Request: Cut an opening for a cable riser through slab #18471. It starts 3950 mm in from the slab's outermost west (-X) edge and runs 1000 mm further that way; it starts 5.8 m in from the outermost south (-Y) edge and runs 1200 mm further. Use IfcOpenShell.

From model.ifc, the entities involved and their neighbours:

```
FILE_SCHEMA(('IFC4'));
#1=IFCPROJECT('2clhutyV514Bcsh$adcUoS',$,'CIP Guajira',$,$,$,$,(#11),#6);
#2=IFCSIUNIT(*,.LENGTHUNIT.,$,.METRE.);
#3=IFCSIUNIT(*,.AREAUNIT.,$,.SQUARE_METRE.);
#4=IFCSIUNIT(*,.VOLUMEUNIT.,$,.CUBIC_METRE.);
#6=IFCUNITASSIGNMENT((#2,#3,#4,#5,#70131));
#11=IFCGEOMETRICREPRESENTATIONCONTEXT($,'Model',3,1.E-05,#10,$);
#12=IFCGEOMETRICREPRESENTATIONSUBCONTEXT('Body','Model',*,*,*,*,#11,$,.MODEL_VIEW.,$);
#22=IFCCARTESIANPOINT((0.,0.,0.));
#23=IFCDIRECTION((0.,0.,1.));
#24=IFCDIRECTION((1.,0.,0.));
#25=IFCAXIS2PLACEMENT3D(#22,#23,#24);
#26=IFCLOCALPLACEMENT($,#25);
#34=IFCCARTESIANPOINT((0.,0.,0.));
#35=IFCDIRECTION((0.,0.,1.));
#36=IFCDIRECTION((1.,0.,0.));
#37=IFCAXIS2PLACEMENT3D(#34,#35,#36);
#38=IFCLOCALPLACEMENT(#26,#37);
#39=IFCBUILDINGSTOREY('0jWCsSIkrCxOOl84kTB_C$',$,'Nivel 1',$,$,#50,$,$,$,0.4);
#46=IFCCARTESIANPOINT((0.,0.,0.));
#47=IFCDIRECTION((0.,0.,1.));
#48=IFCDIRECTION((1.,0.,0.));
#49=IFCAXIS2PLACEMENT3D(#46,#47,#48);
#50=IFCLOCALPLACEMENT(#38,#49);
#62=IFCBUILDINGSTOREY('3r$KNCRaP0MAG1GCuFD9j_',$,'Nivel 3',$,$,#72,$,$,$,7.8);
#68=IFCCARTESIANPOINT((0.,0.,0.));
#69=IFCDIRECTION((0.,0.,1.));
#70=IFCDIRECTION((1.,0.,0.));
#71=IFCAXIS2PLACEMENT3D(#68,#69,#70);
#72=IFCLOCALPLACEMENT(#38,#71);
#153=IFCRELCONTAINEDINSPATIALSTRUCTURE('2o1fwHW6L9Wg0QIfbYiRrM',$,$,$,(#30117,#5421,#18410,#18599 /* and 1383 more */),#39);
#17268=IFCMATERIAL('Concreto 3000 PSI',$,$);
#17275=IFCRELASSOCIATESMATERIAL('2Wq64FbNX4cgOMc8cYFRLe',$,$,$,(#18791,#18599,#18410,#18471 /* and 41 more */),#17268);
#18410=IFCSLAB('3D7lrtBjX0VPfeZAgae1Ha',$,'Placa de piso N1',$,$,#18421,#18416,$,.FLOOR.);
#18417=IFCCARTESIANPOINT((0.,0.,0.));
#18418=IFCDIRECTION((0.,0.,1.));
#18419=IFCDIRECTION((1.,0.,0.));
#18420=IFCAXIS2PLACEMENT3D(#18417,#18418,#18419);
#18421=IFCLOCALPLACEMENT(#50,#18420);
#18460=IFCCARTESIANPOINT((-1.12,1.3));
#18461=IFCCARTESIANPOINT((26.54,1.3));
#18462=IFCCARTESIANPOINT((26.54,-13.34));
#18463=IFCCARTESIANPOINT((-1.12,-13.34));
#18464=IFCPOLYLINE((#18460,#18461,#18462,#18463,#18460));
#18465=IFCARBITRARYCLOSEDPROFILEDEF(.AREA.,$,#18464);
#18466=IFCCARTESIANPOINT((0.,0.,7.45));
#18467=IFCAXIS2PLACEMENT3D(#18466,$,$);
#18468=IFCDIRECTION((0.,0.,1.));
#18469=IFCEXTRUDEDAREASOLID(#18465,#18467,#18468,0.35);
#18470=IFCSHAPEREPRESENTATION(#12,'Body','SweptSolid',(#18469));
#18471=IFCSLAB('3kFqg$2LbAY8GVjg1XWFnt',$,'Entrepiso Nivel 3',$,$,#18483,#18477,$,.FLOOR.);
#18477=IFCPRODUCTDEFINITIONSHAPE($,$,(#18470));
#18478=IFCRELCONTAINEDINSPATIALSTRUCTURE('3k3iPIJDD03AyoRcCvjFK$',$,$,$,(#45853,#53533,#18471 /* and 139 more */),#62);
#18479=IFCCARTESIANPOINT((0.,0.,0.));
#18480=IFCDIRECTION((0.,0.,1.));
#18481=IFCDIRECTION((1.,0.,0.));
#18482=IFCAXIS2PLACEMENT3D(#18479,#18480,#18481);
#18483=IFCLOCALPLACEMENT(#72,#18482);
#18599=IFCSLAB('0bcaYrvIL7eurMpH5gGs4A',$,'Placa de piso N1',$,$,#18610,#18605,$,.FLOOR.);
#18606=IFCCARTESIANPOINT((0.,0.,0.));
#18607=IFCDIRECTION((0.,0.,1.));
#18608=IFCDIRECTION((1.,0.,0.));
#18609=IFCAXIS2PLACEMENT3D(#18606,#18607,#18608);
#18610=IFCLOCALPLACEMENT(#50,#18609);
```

```python
import numpy as np
import ifcopenshell
import ifcopenshell.api.feature
import ifcopenshell.api.geometry
import ifcopenshell.api.root
import ifcopenshell.geom
import ifcopenshell.util.placement
import ifcopenshell.util.representation
import ifcopenshell.util.shape
import ifcopenshell.util.unit

model = ifcopenshell.open("model.ifc")
unit_scale = ifcopenshell.util.unit.calculate_unit_scale(model)
settings = ifcopenshell.geom.settings()


def volume(element):
    """Net volume in cubic metres, openings subtracted."""
    shape = ifcopenshell.geom.create_shape(settings, element)
    return ifcopenshell.util.shape.get_volume(shape.geometry)


slab = model.by_id(18471)
before = volume(slab)

# Extent in the slab's own axes, in metres. The edges named are its -X and -Y sides.
slab_shape = ifcopenshell.geom.create_shape(settings, slab)
vertices = ifcopenshell.util.shape.get_vertices(slab_shape.geometry)
x_min, y_min, bottom = vertices.min(axis=0)
top = vertices[:, 2].max()

opening = ifcopenshell.api.root.create_entity(model, ifc_class="IfcOpeningElement", name="Cable riser opening", predefined_type="OPENING")
context = ifcopenshell.util.representation.get_context(model, "Model", "Body", "MODEL_VIEW")
width, depth = 1, 1.2
outline = [(0.0, 0.0), (width, 0.0), (width, depth), (0.0, depth), (0.0, 0.0)]
# Overshoot both faces by 50 mm so the cut is clean.
shape = ifcopenshell.api.geometry.add_slab_representation(
    model, context=context, depth=top - bottom + 0.1, polyline=outline
)
ifcopenshell.api.geometry.assign_representation(model, product=opening, representation=shape)

matrix = ifcopenshell.util.placement.get_local_placement(slab.ObjectPlacement)
matrix[:, 3] = matrix @ np.append(np.array([x_min + 3.95, y_min + 5.8, bottom - 0.05]) / unit_scale, 1.0)
ifcopenshell.api.geometry.edit_object_placement(model, product=opening, matrix=matrix, is_si=False)
ifcopenshell.api.feature.add_feature(model, feature=opening, element=slab)

after = volume(slab)

print(f"slab volume {before:.3f} -> {after:.3f} m3")

model.write("model_v2.ifc")
```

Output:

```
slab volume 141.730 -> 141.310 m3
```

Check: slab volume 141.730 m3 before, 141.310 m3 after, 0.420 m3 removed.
